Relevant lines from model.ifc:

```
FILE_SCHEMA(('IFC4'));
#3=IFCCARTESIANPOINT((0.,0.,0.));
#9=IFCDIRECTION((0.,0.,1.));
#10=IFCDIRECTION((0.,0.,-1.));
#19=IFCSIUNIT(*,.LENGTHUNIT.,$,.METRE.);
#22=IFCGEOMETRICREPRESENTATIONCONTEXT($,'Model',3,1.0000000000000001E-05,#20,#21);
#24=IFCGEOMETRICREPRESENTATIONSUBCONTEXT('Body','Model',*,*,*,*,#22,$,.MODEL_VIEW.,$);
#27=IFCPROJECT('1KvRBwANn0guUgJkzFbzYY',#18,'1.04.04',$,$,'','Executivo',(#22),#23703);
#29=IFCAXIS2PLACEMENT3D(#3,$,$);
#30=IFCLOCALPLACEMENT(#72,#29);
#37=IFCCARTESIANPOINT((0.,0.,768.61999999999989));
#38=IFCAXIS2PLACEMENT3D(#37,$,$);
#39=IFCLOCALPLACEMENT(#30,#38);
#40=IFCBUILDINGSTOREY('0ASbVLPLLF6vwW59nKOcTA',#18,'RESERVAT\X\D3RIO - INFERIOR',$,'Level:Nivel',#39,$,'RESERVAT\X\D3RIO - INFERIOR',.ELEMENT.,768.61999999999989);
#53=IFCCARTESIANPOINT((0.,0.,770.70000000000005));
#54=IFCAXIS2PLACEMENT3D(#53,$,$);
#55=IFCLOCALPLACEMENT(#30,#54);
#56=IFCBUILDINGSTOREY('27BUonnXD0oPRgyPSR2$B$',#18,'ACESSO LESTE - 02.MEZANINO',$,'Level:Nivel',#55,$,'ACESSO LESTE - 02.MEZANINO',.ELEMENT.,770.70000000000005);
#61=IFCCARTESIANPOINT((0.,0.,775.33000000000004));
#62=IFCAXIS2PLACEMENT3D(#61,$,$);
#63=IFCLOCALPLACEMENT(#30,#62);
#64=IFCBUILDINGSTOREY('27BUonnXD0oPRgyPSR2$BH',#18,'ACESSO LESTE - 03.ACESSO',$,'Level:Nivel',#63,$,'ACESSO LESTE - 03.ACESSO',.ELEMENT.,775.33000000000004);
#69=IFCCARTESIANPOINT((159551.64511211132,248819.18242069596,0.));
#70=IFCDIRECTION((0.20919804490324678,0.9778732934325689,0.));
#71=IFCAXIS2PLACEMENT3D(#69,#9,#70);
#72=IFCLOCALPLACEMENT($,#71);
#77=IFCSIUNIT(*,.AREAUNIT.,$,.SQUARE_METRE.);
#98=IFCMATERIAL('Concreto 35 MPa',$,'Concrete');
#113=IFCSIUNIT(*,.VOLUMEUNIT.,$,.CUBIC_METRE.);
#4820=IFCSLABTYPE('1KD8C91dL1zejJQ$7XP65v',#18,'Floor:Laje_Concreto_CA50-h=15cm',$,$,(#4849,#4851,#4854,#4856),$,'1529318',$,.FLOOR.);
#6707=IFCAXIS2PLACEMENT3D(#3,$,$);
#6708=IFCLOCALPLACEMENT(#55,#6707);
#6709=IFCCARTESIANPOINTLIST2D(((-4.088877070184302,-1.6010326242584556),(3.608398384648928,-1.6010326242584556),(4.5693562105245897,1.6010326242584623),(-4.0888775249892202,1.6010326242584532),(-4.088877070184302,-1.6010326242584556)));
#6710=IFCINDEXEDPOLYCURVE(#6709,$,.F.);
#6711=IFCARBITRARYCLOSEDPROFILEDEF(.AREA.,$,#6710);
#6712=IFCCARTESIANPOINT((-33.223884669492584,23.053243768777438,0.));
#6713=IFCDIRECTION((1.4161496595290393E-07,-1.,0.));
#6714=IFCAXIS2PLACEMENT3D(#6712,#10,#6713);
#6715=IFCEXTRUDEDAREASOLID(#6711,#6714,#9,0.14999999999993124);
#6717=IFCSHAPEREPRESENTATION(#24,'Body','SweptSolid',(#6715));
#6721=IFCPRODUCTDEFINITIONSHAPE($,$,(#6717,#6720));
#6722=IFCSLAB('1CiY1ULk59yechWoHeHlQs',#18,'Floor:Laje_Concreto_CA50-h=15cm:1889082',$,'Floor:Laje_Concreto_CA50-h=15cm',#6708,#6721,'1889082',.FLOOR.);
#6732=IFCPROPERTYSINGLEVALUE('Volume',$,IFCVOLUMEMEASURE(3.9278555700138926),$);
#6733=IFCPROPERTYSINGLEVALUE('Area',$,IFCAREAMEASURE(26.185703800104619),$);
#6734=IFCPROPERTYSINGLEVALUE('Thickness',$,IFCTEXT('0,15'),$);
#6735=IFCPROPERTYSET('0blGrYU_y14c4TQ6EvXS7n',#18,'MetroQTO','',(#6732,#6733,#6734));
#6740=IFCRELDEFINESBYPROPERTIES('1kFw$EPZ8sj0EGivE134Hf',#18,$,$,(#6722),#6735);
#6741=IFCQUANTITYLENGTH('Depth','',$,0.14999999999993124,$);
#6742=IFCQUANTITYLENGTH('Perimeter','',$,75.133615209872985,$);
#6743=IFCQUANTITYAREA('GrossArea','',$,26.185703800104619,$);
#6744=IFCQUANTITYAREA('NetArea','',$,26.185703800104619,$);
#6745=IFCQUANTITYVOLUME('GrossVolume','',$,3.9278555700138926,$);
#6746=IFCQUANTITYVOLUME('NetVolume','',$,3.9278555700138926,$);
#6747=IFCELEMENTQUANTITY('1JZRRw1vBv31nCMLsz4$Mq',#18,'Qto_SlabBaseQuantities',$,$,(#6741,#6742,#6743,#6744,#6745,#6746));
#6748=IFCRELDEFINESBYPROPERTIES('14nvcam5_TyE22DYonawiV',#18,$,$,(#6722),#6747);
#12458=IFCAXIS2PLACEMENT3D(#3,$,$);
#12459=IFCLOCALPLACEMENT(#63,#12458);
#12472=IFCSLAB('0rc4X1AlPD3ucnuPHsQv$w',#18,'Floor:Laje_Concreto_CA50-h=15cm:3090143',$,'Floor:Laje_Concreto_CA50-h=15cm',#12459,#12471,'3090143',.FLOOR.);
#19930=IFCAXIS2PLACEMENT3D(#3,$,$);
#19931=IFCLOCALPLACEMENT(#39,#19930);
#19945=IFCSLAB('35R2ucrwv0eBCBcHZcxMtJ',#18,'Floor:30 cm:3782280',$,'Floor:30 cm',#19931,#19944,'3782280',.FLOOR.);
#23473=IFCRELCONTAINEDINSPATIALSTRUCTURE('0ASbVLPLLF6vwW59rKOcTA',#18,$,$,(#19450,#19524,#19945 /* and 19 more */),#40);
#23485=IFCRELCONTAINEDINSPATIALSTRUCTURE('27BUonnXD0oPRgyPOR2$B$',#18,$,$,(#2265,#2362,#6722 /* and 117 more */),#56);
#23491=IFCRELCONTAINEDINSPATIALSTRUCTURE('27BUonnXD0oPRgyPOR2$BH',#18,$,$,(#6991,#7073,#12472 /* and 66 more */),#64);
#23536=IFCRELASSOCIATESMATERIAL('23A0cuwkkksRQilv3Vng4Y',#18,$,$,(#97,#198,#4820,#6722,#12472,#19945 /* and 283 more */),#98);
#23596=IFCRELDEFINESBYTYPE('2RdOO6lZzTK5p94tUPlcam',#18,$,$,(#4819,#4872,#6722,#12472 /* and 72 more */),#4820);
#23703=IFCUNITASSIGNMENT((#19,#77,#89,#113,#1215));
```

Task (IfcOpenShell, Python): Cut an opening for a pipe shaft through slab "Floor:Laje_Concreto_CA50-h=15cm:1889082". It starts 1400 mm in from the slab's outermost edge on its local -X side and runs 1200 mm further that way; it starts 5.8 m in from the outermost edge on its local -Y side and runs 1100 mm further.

```python
import numpy as np
import ifcopenshell
import ifcopenshell.api.feature
import ifcopenshell.api.geometry
import ifcopenshell.api.pset
import ifcopenshell.api.root
import ifcopenshell.geom
import ifcopenshell.util.element
import ifcopenshell.util.placement
import ifcopenshell.util.representation
import ifcopenshell.util.shape
import ifcopenshell.util.unit

model = ifcopenshell.open("model.ifc")
unit_scale = ifcopenshell.util.unit.calculate_unit_scale(model)
area_scale = ifcopenshell.util.unit.calculate_unit_scale(model, "AREAUNIT")
volume_scale = ifcopenshell.util.unit.calculate_unit_scale(model, "VOLUMEUNIT")
settings = ifcopenshell.geom.settings()


def volume(element):
    """Net volume in cubic metres, openings subtracted."""
    shape = ifcopenshell.geom.create_shape(settings, element)
    return ifcopenshell.util.shape.get_volume(shape.geometry)


slab = model.by_guid("1CiY1ULk59yechWoHeHlQs")
before = volume(slab)

# Extent in the slab's own axes, in metres. The edges named are its -X and -Y sides.
slab_shape = ifcopenshell.geom.create_shape(settings, slab)
vertices = ifcopenshell.util.shape.get_vertices(slab_shape.geometry)
x_min, y_min, bottom = vertices.min(axis=0)
top = vertices[:, 2].max()

opening = ifcopenshell.api.root.create_entity(model, ifc_class="IfcOpeningElement", name="Pipe shaft opening", predefined_type="OPENING")
context = ifcopenshell.util.representation.get_context(model, "Model", "Body", "MODEL_VIEW")
width, depth = 1.2, 1.1
outline = [(0.0, 0.0), (width, 0.0), (width, depth), (0.0, depth), (0.0, 0.0)]
# Overshoot both faces by 50 mm so the cut is clean.
shape = ifcopenshell.api.geometry.add_slab_representation(
    model, context=context, depth=top - bottom + 0.1, polyline=outline
)
ifcopenshell.api.geometry.assign_representation(model, product=opening, representation=shape)

matrix = ifcopenshell.util.placement.get_local_placement(slab.ObjectPlacement)
matrix[:, 3] = matrix @ np.append(np.array([x_min + 1.4, y_min + 5.8, bottom - 0.05]) / unit_scale, 1.0)
ifcopenshell.api.geometry.edit_object_placement(model, product=opening, matrix=matrix, is_si=False)
ifcopenshell.api.feature.add_feature(model, feature=opening, element=slab)

after = volume(slab)

# Update the slab's stored quantities.
pset = model.by_id(ifcopenshell.util.element.get_pset(slab, "MetroQTO", should_inherit=False)["id"])
ifcopenshell.api.pset.edit_pset(model, pset=pset, properties={
    "Volume": model.create_entity("IfcVolumeMeasure", after / volume_scale),
    "Area": model.create_entity("IfcAreaMeasure", after / (top - bottom) / area_scale),
})
qto = model.by_id(ifcopenshell.util.element.get_pset(slab, "Qto_SlabBaseQuantities", should_inherit=False)["id"])
ifcopenshell.api.pset.edit_qto(model, qto=qto, properties={
    "NetArea": after / (top - bottom) / area_scale,
    "NetVolume": after / volume_scale,
})

print(f"slab volume {before:.3f} -> {after:.3f} m3")

model.write("model_rev.ifc")
```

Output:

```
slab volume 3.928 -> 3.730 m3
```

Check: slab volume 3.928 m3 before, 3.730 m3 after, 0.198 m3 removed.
